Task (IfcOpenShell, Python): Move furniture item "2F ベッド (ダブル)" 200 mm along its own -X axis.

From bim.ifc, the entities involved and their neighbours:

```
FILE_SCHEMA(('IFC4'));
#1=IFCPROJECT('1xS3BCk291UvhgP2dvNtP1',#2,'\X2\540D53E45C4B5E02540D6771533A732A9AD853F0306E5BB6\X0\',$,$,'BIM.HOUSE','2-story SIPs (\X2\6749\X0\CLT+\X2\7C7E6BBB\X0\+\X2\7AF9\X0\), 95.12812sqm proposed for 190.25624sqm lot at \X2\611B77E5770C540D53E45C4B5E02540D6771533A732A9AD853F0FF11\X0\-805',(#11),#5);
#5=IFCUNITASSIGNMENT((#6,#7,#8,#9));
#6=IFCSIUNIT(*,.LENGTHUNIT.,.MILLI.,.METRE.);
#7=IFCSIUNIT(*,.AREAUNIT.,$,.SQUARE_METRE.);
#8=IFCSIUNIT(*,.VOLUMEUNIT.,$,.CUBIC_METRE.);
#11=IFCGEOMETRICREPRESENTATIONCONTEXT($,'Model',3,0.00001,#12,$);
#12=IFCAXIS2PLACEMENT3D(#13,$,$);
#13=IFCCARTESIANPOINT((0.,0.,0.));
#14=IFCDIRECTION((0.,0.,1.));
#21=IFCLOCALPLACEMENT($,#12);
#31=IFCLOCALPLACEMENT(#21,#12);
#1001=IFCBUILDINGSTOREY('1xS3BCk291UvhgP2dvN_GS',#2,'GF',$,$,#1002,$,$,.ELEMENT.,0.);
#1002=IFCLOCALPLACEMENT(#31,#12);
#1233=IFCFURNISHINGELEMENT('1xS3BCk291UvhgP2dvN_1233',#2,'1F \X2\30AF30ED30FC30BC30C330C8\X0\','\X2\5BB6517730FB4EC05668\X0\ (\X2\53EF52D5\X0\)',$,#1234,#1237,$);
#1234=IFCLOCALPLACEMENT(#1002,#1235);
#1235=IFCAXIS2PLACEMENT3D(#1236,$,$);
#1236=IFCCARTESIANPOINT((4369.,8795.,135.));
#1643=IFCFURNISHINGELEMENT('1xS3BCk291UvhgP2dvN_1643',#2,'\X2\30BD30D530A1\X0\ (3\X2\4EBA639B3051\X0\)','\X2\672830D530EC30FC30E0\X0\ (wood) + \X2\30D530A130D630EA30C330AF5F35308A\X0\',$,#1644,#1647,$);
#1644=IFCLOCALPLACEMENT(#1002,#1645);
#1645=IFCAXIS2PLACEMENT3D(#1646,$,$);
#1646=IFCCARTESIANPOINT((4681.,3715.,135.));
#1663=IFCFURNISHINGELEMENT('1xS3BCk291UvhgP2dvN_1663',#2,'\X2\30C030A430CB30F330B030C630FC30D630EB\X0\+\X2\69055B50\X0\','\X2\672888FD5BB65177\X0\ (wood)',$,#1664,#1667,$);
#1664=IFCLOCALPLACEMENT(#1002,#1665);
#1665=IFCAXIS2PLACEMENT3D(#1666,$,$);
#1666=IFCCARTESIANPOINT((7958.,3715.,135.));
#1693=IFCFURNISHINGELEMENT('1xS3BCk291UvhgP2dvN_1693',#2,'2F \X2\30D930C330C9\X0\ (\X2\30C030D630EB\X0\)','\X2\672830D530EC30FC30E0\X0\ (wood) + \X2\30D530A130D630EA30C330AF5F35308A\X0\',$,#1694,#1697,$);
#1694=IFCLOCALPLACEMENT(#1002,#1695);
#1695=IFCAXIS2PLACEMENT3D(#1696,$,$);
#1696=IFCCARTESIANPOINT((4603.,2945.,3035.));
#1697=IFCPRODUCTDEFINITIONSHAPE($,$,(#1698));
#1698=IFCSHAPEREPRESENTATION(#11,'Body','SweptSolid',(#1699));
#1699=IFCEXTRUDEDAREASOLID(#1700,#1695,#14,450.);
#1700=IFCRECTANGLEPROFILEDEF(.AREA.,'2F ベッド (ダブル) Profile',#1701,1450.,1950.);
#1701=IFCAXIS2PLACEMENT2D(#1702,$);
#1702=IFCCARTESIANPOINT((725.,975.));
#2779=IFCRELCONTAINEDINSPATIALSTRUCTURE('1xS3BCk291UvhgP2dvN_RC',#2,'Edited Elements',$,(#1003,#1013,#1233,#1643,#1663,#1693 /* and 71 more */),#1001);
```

```python
import ifcopenshell
import ifcopenshell.api.geometry
import ifcopenshell.util.placement
import ifcopenshell.util.unit

model = ifcopenshell.open("bim.ifc")
unit_scale = ifcopenshell.util.unit.calculate_unit_scale(model)

item = model.by_guid("1xS3BCk291UvhgP2dvN_1693")
matrix = ifcopenshell.util.placement.get_local_placement(item.ObjectPlacement)
matrix[:3, 3] -= matrix[:3, 0] * 0.2 / unit_scale
ifcopenshell.api.geometry.edit_object_placement(model, product=item, matrix=matrix, is_si=False)

print(ifcopenshell.util.placement.get_local_placement(item.ObjectPlacement).round(3) + 0.0)

model.write("bim_edited.ifc")
```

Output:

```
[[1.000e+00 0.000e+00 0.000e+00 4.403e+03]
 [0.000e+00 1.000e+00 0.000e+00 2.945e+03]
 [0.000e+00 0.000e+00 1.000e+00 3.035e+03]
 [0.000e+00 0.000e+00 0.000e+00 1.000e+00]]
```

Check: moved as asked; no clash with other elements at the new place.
